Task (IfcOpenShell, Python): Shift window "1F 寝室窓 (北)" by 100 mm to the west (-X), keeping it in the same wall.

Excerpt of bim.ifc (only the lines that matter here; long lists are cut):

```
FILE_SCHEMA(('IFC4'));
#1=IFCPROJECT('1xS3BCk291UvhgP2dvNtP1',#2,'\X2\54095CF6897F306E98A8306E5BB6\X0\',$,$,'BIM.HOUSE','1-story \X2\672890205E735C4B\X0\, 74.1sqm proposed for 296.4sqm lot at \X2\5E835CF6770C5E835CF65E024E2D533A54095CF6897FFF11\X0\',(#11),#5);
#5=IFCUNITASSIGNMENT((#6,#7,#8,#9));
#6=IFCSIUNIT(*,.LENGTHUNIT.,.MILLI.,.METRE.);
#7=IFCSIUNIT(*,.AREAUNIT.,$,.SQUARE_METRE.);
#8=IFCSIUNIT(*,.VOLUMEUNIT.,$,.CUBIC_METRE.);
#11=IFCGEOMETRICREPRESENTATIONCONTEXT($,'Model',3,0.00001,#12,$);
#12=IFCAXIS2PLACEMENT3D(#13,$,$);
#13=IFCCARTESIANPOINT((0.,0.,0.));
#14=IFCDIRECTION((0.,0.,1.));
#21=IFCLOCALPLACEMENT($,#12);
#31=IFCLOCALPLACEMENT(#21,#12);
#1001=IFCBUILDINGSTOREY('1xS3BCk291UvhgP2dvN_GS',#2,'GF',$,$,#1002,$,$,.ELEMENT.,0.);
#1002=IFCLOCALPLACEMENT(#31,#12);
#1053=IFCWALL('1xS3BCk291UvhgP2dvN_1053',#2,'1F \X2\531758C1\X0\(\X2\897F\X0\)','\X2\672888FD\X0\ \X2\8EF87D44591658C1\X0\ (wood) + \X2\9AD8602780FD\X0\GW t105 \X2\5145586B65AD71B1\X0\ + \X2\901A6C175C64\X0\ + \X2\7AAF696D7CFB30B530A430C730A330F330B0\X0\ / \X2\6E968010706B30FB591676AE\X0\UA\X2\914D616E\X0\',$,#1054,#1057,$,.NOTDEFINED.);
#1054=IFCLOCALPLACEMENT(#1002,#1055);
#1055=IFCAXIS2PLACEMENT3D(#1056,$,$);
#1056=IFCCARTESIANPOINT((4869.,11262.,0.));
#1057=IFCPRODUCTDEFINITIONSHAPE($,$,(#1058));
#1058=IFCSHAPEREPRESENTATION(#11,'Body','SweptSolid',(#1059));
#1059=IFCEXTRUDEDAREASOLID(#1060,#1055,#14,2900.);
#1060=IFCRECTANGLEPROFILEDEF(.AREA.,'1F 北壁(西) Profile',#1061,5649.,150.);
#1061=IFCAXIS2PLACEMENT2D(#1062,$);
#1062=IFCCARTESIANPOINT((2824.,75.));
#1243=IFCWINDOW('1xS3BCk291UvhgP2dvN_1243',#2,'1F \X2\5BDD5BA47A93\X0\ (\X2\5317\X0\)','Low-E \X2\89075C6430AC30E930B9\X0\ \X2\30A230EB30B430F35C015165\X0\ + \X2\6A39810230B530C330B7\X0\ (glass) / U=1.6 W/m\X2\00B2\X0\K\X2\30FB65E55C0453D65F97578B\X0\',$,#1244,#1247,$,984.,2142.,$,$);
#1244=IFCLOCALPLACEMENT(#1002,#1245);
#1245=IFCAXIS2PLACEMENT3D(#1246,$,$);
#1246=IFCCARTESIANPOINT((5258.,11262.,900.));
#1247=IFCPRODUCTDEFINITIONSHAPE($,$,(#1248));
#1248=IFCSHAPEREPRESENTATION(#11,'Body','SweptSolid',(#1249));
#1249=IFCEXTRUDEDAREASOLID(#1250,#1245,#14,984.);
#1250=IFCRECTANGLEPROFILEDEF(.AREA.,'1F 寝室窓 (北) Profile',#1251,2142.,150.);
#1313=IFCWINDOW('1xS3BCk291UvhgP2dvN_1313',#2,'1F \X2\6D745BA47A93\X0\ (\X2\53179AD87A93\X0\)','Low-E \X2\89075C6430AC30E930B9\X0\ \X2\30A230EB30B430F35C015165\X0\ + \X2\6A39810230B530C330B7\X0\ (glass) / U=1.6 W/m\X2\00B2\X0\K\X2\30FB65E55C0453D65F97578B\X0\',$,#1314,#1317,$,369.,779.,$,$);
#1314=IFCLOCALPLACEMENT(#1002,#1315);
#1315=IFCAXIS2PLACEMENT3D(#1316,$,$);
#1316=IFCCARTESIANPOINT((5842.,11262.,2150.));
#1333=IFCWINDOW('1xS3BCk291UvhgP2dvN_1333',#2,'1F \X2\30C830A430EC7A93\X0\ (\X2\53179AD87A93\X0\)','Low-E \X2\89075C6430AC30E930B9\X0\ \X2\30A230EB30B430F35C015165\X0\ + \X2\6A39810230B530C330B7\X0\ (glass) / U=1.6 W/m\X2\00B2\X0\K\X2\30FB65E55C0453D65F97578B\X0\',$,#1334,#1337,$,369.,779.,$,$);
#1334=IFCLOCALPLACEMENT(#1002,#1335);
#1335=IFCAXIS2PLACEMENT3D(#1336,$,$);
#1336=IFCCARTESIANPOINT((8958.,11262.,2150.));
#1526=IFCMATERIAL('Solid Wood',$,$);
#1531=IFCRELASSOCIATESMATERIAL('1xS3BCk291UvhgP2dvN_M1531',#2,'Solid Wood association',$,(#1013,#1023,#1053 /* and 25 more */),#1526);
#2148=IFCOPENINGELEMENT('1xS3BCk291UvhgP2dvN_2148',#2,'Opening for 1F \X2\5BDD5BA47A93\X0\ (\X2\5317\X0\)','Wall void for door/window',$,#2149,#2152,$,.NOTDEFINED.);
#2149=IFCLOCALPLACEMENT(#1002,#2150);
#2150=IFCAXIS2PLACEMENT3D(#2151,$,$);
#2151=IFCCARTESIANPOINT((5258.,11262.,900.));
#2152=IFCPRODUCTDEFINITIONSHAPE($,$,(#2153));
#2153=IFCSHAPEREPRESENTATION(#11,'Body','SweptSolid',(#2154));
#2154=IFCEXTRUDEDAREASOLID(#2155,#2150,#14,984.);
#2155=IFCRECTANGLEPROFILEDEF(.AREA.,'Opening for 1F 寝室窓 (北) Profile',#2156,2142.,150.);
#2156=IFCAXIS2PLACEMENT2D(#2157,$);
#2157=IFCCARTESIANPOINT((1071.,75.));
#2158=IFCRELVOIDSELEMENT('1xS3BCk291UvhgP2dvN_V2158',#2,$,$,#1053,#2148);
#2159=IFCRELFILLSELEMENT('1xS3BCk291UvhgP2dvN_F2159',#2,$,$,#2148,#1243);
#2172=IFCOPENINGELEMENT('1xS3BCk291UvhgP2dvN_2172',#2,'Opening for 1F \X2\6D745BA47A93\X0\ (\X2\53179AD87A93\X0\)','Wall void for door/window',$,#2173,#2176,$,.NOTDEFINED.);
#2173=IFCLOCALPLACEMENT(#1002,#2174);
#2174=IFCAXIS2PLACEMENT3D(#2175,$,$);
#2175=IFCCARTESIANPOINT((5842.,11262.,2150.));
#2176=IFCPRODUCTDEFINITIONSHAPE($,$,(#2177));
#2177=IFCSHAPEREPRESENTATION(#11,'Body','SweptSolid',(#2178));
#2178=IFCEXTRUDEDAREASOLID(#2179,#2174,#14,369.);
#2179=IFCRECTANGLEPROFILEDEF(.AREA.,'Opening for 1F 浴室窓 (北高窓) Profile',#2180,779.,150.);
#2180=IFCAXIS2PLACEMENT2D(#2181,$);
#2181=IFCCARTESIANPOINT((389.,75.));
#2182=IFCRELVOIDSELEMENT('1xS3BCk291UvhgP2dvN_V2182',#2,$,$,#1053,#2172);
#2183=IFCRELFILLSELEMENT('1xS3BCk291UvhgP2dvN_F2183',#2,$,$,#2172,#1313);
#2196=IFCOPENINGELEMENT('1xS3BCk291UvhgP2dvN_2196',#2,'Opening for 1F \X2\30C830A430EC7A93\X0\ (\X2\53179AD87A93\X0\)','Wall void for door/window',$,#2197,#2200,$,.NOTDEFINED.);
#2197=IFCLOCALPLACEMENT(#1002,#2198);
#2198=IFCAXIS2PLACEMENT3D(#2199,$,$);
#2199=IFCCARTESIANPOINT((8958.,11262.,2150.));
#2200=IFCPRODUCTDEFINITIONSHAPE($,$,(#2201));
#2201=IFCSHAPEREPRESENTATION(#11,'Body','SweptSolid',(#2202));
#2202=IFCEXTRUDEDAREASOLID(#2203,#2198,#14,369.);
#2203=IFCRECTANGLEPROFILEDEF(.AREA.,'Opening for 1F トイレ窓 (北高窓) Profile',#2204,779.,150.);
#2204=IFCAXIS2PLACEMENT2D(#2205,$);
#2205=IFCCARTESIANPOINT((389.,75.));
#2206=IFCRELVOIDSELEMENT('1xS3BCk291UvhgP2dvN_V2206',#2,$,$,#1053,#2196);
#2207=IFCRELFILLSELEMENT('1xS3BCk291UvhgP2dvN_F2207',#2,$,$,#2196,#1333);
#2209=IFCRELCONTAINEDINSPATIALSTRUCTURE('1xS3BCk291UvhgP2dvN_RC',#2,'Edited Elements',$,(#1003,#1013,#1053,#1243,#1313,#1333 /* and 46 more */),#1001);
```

```python
import ifcopenshell
import ifcopenshell.api.geometry
import ifcopenshell.util.placement

model = ifcopenshell.open("bim.ifc")

window = model.by_id(1243)
opening = window.FillsVoids[0].RelatingOpeningElement
wall = opening.VoidsElements[0].RelatingBuildingElement

wall_matrix = ifcopenshell.util.placement.get_local_placement(wall.ObjectPlacement)
shift = wall_matrix[:3, 0] * -100.0
before = ifcopenshell.util.placement.get_local_placement(window.ObjectPlacement)[:3, 3].copy()

# The window is not placed relative to its opening, so move both.
for product in (opening, window):
    matrix = ifcopenshell.util.placement.get_local_placement(product.ObjectPlacement)
    matrix[:3, 3] += shift
    ifcopenshell.api.geometry.edit_object_placement(model, product=product, matrix=matrix, is_si=False)

after = ifcopenshell.util.placement.get_local_placement(window.ObjectPlacement)[:3, 3]
print("window moved by", (after - before).round(3) + 0.0)

model.write("bim_rev.ifc")
```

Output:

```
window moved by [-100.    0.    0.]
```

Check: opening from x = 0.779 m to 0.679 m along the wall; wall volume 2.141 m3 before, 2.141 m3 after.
